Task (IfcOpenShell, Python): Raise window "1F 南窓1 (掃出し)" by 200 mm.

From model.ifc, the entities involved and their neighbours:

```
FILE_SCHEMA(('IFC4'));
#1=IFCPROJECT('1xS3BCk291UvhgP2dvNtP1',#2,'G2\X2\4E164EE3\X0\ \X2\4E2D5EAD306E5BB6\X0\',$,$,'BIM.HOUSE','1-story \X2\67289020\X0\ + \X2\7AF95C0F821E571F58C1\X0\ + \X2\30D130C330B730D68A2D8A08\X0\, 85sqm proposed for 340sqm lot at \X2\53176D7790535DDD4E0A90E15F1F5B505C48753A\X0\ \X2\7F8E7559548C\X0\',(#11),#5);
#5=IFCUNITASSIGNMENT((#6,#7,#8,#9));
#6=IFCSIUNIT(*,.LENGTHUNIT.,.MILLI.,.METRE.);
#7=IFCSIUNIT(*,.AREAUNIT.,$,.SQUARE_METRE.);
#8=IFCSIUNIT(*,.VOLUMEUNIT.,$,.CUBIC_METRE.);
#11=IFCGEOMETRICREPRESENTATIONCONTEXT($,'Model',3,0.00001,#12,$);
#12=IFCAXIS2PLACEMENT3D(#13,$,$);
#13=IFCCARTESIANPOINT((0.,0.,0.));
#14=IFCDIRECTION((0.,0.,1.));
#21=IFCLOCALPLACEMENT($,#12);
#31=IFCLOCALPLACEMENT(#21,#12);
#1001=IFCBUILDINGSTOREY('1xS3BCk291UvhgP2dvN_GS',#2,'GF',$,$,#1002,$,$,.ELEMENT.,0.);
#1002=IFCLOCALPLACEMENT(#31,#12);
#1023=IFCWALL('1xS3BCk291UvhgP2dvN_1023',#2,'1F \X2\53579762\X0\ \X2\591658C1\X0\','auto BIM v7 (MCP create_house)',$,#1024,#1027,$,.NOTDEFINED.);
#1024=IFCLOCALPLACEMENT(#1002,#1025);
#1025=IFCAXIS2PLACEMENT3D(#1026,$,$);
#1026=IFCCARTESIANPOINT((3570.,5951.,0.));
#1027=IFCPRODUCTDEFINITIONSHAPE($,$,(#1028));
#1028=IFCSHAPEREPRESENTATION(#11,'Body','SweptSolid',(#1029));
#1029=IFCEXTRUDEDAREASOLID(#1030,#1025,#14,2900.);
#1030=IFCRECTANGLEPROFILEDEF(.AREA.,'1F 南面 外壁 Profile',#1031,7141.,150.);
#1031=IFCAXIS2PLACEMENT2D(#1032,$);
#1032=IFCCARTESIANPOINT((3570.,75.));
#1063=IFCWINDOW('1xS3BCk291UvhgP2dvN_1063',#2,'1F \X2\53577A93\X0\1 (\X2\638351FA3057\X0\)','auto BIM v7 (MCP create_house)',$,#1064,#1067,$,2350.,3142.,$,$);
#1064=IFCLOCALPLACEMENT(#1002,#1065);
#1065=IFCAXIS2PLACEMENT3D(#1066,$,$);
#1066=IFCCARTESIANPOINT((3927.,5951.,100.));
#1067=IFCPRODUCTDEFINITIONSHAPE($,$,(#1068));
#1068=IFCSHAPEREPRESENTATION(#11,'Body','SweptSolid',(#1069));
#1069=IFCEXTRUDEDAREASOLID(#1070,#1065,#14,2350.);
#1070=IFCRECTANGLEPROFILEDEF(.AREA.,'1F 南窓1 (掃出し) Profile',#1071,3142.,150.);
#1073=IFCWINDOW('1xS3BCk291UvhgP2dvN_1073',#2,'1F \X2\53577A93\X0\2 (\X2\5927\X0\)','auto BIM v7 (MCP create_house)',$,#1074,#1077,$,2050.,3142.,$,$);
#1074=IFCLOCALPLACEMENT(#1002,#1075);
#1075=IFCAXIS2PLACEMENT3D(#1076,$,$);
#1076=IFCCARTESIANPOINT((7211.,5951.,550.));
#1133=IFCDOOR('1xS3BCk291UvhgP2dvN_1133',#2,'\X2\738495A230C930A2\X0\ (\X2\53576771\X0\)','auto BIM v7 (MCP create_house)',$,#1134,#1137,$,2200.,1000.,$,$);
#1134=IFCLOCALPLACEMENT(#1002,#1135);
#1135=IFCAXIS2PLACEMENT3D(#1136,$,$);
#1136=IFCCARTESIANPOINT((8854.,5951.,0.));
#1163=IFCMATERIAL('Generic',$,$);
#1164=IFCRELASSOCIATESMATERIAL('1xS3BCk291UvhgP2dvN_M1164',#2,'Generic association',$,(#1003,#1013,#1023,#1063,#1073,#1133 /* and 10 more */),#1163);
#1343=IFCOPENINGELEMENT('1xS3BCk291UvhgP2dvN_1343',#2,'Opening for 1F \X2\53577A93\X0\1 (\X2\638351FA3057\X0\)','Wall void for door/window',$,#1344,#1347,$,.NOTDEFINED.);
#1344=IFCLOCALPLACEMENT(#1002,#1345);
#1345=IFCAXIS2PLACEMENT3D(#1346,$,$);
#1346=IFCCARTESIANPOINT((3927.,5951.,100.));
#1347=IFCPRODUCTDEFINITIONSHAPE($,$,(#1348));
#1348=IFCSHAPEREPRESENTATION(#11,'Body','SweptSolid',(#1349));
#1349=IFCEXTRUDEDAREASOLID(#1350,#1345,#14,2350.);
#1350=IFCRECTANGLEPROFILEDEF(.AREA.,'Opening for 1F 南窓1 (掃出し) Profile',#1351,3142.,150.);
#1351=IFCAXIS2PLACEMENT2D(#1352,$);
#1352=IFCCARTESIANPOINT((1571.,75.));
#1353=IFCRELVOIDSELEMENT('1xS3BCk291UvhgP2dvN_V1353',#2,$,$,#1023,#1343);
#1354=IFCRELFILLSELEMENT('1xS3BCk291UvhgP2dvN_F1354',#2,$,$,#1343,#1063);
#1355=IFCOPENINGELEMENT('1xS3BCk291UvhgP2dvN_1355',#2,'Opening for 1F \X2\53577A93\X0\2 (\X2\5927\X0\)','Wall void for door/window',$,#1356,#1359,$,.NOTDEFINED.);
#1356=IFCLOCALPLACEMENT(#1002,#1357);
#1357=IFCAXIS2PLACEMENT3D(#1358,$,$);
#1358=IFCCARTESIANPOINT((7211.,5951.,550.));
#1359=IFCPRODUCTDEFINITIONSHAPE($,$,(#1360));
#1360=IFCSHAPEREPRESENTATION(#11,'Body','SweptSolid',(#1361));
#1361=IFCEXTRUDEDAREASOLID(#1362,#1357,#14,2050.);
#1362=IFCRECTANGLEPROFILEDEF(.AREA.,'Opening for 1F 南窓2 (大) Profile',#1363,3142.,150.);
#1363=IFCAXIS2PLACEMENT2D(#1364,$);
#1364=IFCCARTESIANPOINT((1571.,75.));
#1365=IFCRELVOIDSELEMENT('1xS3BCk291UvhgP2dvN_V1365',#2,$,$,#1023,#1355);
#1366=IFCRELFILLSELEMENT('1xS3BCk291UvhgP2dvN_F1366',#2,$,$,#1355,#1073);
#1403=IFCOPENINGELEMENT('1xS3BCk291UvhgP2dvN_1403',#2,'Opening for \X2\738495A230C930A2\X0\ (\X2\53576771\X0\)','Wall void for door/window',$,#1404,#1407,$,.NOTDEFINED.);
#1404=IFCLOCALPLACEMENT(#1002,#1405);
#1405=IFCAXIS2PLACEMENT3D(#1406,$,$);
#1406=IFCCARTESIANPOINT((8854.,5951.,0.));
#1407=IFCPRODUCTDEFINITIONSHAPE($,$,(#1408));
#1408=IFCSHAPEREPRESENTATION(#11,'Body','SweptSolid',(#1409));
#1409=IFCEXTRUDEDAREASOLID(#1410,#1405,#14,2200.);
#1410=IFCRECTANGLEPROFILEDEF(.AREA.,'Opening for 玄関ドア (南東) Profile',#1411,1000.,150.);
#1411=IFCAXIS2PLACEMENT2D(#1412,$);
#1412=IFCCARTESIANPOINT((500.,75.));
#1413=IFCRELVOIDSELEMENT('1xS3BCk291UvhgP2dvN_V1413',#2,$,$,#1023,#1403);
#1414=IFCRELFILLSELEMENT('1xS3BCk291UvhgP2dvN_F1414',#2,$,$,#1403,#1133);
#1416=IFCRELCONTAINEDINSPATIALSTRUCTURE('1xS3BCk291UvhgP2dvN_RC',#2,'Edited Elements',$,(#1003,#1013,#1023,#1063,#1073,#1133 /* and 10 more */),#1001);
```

```python
import numpy as np
import ifcopenshell
import ifcopenshell.api.geometry
import ifcopenshell.util.placement
import ifcopenshell.util.unit

model = ifcopenshell.open("model.ifc")
unit_scale = ifcopenshell.util.unit.calculate_unit_scale(model)

window = model.by_id(1063)
opening = window.FillsVoids[0].RelatingOpeningElement
dz = 200.0

shift = np.array([0.0, 0.0, dz])
# The window is not placed relative to its opening, so move both.
for product in (opening, window):
    matrix = ifcopenshell.util.placement.get_local_placement(product.ObjectPlacement)
    matrix[:3, 3] += shift
    ifcopenshell.api.geometry.edit_object_placement(model, product=product, matrix=matrix, is_si=False)

print(f"moved by {dz * unit_scale:+.3f} m")

model.write("model-out.ifc")
```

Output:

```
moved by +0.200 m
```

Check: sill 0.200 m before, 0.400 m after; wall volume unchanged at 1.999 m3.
